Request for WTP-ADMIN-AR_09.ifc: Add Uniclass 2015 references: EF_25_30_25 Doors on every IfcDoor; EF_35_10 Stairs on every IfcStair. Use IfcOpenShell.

First a look at what the model holds.

```python
import ifcopenshell

model = ifcopenshell.open("WTP-ADMIN-AR_09.ifc")
print(model.schema)
print("classifications:", [c.Name for c in model.by_type("IfcClassification")])
for ifc_class in ("IfcDoor", "IfcRoof", "IfcStair", "IfcWall", "IfcWindow"):
    print(ifc_class, len(model.by_type(ifc_class)))
```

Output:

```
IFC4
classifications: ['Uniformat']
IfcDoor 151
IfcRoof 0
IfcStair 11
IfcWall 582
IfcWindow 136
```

```python
import ifcopenshell
import ifcopenshell.api.classification

model = ifcopenshell.open("WTP-ADMIN-AR_09.ifc")

system = ifcopenshell.api.classification.add_classification(model, classification="Uniclass 2015")

codes = {
    "IfcDoor": ("EF_25_30_25", "Doors"),
    "IfcStair": ("EF_35_10", "Stairs"),
}
for ifc_class, (code, name) in codes.items():
    products = model.by_type(ifc_class)
    ifcopenshell.api.classification.add_reference(
        model, products=products, classification=system, identification=code, name=name
    )
    print(code, len(products))

model.write("WTP-ADMIN-AR_09_updated.ifc")
```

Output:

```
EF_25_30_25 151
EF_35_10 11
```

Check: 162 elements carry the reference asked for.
